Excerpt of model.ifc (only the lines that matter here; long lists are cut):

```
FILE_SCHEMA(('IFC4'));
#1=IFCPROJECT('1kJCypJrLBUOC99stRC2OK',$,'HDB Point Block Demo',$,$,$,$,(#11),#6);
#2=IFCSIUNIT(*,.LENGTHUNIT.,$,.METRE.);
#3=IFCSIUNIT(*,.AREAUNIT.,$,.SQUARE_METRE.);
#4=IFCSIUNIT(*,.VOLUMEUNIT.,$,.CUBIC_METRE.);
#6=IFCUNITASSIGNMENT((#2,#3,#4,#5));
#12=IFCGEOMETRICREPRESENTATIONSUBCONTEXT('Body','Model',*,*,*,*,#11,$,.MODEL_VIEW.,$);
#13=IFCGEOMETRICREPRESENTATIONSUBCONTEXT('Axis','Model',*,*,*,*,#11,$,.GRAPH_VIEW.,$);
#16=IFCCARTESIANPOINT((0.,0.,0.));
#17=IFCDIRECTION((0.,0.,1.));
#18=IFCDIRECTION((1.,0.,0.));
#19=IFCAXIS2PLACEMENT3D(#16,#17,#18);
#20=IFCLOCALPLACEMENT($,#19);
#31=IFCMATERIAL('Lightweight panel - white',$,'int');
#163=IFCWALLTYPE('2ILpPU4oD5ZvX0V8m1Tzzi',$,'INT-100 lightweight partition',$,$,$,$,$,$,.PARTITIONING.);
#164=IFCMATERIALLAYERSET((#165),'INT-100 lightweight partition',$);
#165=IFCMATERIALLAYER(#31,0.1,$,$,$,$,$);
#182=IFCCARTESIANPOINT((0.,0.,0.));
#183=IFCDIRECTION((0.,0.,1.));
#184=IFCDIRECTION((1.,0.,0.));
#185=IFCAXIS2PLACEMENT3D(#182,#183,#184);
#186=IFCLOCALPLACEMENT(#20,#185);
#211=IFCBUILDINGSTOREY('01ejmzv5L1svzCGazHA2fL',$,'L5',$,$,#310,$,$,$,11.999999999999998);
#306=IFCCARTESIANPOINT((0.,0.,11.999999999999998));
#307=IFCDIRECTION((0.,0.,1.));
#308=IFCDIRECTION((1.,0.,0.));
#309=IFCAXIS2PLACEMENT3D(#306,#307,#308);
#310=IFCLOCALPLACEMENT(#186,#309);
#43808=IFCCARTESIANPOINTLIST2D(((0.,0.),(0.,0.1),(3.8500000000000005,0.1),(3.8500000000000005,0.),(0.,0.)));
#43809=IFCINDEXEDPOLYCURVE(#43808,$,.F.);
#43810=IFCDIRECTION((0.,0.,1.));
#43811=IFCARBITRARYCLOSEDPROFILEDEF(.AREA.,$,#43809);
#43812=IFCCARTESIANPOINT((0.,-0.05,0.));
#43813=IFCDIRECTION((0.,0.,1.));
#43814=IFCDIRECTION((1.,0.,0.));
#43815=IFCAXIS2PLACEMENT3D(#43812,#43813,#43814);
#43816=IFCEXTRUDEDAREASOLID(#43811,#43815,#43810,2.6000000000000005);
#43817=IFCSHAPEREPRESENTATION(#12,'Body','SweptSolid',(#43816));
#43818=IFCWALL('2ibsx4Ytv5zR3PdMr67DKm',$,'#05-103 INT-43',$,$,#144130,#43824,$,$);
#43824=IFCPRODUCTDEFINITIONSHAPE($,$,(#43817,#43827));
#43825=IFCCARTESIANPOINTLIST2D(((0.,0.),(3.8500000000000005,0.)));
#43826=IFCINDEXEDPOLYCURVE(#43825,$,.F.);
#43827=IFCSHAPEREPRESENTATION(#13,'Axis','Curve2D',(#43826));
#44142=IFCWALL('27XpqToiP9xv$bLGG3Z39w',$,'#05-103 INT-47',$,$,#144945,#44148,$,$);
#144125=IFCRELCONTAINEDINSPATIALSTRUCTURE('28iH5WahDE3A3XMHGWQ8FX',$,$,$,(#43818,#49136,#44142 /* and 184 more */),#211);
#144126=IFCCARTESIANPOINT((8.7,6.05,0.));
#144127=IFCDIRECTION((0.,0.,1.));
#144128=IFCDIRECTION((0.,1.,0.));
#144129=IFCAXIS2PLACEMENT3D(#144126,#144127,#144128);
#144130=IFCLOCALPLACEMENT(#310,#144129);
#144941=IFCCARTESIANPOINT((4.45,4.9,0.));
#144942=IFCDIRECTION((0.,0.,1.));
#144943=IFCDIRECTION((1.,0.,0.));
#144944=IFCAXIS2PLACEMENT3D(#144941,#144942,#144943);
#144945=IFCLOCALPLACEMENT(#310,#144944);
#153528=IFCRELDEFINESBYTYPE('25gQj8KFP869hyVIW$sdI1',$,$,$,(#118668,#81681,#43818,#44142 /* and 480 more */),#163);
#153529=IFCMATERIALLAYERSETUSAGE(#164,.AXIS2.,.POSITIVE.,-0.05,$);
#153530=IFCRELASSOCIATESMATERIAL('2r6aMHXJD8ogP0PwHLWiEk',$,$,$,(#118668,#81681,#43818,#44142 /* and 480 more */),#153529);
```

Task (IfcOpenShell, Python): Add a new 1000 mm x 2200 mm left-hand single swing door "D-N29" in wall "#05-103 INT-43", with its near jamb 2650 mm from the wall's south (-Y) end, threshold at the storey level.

```python
import numpy as np
import ifcopenshell
import ifcopenshell.api.feature
import ifcopenshell.api.geometry
import ifcopenshell.api.root
import ifcopenshell.api.spatial
import ifcopenshell.geom
import ifcopenshell.util.element
import ifcopenshell.util.placement
import ifcopenshell.util.representation
import ifcopenshell.util.shape
import ifcopenshell.util.unit

model = ifcopenshell.open("model.ifc")
unit_scale = ifcopenshell.util.unit.calculate_unit_scale(model)
settings = ifcopenshell.geom.settings()


def volume(element):
    """Net volume in cubic metres, openings subtracted."""
    shape = ifcopenshell.geom.create_shape(settings, element)
    return ifcopenshell.util.shape.get_volume(shape.geometry)


wall = model.by_id(43818)
storey = ifcopenshell.util.element.get_container(wall, ifc_class="IfcBuildingStorey")
context = ifcopenshell.util.representation.get_context(model, "Model", "Body", "MODEL_VIEW")
before = volume(wall)

width, height, from_end, sill = 1, 2.2, 2.65, 0.0  # metres

# The wall runs along its own X axis, and the end named is its -X end.
wall_shape = ifcopenshell.geom.create_shape(settings, wall)
x, y, z = ifcopenshell.util.shape.get_vertices(wall_shape.geometry).T
start = x.min() + from_end
face, thickness = float(y.min()), float(y.max() - y.min())
wall_matrix = ifcopenshell.util.placement.get_local_placement(wall.ObjectPlacement)
level = ifcopenshell.util.placement.get_local_placement(storey.ObjectPlacement)[2, 3]


def in_wall(x, y):
    """Placement at x, y metres in the wall's axes, at sill height."""
    matrix = wall_matrix.copy()
    matrix[:, 3] = wall_matrix @ np.array([x / unit_scale, y / unit_scale, 0.0, 1.0])
    matrix[2, 3] = level + sill / unit_scale
    return matrix


# Opening: a box that overshoots both wall faces by 50 mm.
opening = ifcopenshell.api.root.create_entity(model, ifc_class="IfcOpeningElement", predefined_type="OPENING")
box = ifcopenshell.api.geometry.add_wall_representation(
    model, context=context, length=width, height=height, thickness=thickness + 0.1
)
ifcopenshell.api.geometry.assign_representation(model, product=opening, representation=box)
ifcopenshell.api.geometry.edit_object_placement(model, product=opening, matrix=in_wall(start, face - 0.05), is_si=False)
ifcopenshell.api.feature.add_feature(model, feature=opening, element=wall)

door = ifcopenshell.api.root.create_entity(model, ifc_class="IfcDoor", name="D-N29", predefined_type="DOOR")
door.OverallWidth, door.OverallHeight = width / unit_scale, height / unit_scale
door.OperationType = "SINGLE_SWING_LEFT"
body = ifcopenshell.api.geometry.add_door_representation(
    model,
    context=context,
    overall_width=door.OverallWidth,
    overall_height=door.OverallHeight,
    operation_type="SINGLE_SWING_LEFT",
    lining_properties={"LiningDepth": thickness / unit_scale, "ThresholdDepth": thickness / unit_scale},
)
ifcopenshell.api.geometry.assign_representation(model, product=door, representation=body)
ifcopenshell.api.spatial.assign_container(model, products=[door], relating_structure=storey)
ifcopenshell.api.feature.add_filling(model, opening=opening, element=door)

# The lining spans the wall, so the door starts at the wall face.
ifcopenshell.api.geometry.edit_object_placement(model, product=door, matrix=in_wall(start, face), is_si=False)

after = volume(wall)

print(f"wall volume {before:.3f} -> {after:.3f} m3")

model.write("model_v2.ifc")
```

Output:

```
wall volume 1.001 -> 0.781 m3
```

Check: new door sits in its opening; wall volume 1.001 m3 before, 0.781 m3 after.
